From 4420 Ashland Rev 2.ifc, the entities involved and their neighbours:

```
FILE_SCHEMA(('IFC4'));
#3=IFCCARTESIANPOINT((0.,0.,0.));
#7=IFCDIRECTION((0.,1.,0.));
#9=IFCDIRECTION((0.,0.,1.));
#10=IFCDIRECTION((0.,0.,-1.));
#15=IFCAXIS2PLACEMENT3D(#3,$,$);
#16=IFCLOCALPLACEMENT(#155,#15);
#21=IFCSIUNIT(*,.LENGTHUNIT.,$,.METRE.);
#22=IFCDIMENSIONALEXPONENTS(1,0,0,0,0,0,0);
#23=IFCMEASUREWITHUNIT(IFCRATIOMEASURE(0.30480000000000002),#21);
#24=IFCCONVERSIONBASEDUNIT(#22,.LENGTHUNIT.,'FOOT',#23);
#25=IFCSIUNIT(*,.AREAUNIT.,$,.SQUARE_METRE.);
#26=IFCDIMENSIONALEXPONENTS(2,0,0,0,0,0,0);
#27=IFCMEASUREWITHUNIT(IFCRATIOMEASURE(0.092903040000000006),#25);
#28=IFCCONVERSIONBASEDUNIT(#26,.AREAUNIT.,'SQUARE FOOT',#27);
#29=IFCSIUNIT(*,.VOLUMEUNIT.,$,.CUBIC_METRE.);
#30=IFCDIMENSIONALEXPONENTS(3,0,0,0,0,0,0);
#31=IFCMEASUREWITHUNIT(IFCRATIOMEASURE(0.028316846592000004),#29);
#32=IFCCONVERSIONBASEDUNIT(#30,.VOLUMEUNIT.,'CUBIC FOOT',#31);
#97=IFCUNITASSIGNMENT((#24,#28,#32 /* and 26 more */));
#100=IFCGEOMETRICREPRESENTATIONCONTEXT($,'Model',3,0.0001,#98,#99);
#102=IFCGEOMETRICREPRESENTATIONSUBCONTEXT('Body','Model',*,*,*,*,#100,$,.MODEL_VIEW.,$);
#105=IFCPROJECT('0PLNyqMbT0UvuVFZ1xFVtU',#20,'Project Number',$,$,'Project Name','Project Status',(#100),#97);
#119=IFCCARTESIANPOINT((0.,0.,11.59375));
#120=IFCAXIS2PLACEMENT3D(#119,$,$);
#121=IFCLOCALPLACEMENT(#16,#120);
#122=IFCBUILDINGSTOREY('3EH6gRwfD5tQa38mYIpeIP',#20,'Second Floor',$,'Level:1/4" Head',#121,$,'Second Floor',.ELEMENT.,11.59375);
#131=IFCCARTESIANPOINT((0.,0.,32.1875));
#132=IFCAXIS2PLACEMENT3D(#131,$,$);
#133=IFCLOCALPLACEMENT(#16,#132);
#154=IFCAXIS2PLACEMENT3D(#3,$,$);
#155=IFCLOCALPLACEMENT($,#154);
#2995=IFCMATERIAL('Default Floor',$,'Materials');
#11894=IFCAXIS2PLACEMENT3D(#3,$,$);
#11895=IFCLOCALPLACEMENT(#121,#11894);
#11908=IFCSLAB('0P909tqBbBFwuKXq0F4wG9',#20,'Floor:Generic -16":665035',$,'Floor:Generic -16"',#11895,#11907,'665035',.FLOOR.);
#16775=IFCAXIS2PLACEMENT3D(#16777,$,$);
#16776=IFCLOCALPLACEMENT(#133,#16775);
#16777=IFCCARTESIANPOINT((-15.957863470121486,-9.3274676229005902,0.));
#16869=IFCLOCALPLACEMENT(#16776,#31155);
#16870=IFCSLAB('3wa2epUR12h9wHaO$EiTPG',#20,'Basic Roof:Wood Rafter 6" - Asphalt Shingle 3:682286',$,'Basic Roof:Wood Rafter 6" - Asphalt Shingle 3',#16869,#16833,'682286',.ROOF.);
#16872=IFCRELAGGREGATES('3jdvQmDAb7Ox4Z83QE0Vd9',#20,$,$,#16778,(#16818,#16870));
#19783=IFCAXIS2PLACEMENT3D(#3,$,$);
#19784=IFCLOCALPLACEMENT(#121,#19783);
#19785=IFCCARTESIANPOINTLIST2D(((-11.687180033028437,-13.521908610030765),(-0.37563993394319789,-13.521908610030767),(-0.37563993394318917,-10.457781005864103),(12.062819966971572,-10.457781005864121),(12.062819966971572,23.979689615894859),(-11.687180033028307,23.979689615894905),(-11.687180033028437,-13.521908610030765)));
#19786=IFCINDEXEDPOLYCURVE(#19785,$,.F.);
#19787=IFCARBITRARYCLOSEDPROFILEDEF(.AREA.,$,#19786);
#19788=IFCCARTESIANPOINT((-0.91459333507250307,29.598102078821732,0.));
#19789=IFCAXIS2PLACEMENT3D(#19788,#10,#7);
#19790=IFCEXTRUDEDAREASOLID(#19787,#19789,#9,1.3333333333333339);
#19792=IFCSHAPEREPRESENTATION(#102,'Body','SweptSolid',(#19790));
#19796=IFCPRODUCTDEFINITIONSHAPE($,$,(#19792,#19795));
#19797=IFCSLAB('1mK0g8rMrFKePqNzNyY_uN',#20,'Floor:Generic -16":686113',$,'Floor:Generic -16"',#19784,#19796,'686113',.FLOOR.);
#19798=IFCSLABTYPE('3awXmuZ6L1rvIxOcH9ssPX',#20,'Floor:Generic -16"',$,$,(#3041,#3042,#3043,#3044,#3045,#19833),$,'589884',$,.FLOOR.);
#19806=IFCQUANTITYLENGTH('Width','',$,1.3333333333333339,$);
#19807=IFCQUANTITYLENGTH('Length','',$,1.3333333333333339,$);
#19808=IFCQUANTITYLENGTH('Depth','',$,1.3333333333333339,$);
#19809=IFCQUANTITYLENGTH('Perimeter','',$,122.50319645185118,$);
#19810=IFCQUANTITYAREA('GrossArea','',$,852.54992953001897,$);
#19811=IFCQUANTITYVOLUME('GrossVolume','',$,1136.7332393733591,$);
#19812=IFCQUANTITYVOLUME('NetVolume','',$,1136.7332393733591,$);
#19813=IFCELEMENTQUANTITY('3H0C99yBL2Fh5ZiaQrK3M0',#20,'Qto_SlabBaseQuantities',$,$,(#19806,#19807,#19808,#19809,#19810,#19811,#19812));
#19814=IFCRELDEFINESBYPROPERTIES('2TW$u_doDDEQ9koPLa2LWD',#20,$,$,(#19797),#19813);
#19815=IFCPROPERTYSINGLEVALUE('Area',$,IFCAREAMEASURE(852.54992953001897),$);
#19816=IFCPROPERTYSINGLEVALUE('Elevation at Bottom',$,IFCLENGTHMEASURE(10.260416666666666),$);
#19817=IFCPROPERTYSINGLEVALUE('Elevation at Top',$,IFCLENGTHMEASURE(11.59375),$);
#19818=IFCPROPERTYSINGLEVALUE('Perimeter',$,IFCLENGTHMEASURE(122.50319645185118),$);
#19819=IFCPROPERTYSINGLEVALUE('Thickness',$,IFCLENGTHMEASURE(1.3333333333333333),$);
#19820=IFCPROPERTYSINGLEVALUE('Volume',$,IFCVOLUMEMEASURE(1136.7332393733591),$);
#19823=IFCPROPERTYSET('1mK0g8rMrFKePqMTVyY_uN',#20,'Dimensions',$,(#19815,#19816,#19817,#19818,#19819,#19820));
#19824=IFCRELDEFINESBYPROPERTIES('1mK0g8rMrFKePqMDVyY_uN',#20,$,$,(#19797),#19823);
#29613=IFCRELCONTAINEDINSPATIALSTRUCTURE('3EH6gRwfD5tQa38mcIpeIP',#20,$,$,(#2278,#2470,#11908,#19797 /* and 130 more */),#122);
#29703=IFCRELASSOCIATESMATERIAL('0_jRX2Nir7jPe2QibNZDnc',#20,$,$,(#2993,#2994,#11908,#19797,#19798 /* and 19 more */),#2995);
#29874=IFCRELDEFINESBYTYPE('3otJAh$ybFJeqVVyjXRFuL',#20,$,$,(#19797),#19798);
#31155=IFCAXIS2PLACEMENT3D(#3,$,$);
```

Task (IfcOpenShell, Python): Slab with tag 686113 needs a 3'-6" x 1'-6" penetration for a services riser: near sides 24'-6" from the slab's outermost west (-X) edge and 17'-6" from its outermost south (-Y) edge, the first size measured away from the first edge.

```python
import numpy as np
import ifcopenshell
import ifcopenshell.api.feature
import ifcopenshell.api.geometry
import ifcopenshell.api.pset
import ifcopenshell.api.root
import ifcopenshell.geom
import ifcopenshell.util.element
import ifcopenshell.util.placement
import ifcopenshell.util.representation
import ifcopenshell.util.shape
import ifcopenshell.util.unit

model = ifcopenshell.open("4420 Ashland Rev 2.ifc")
unit_scale = ifcopenshell.util.unit.calculate_unit_scale(model)
area_scale = ifcopenshell.util.unit.calculate_unit_scale(model, "AREAUNIT")
volume_scale = ifcopenshell.util.unit.calculate_unit_scale(model, "VOLUMEUNIT")
settings = ifcopenshell.geom.settings()


def volume(element):
    """Net volume in cubic metres, openings subtracted."""
    shape = ifcopenshell.geom.create_shape(settings, element)
    return ifcopenshell.util.shape.get_volume(shape.geometry)


slab = model.by_guid("1mK0g8rMrFKePqNzNyY_uN")
before = volume(slab)

# Extent in the slab's own axes, in metres. The edges named are its -X and -Y sides.
slab_shape = ifcopenshell.geom.create_shape(settings, slab)
vertices = ifcopenshell.util.shape.get_vertices(slab_shape.geometry)
x_min, y_min, bottom = vertices.min(axis=0)
top = vertices[:, 2].max()

opening = ifcopenshell.api.root.create_entity(model, ifc_class="IfcOpeningElement", name="Services riser opening", predefined_type="OPENING")
context = ifcopenshell.util.representation.get_context(model, "Model", "Body", "MODEL_VIEW")
width, depth = 1.0668, 0.4572
outline = [(0.0, 0.0), (width, 0.0), (width, depth), (0.0, depth), (0.0, 0.0)]
# Overshoot both faces by 50 mm so the cut is clean.
shape = ifcopenshell.api.geometry.add_slab_representation(
    model, context=context, depth=top - bottom + 0.1, polyline=outline
)
ifcopenshell.api.geometry.assign_representation(model, product=opening, representation=shape)

matrix = ifcopenshell.util.placement.get_local_placement(slab.ObjectPlacement)
matrix[:, 3] = matrix @ np.append(np.array([x_min + 7.4676, y_min + 5.334, bottom - 0.05]) / unit_scale, 1.0)
ifcopenshell.api.geometry.edit_object_placement(model, product=opening, matrix=matrix, is_si=False)
ifcopenshell.api.feature.add_feature(model, feature=opening, element=slab)

after = volume(slab)

# Update the slab's stored quantities.
qto = model.by_id(ifcopenshell.util.element.get_pset(slab, "Qto_SlabBaseQuantities", should_inherit=False)["id"])
ifcopenshell.api.pset.edit_qto(model, qto=qto, properties={"NetVolume": after / volume_scale})
pset = model.by_id(ifcopenshell.util.element.get_pset(slab, "Dimensions", should_inherit=False)["id"])
ifcopenshell.api.pset.edit_pset(model, pset=pset, properties={
    "Area": model.create_entity("IfcAreaMeasure", after / (top - bottom) / area_scale),
    "Volume": model.create_entity("IfcVolumeMeasure", after / volume_scale),
})

print(f"slab volume {before:.3f} -> {after:.3f} m3")

model.write("4420 Ashland Rev 2_updated.ifc")
```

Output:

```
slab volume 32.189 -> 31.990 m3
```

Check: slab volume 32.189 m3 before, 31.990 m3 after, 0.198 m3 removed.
